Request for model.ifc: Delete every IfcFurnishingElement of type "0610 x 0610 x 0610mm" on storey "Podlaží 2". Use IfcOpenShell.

First a look at what the model holds.

```python
import ifcopenshell
import ifcopenshell.util.element

model = ifcopenshell.open("model.ifc")
print(model.schema)
storey = next(s for s in model.by_type("IfcBuildingStorey") if s.Name == "Podlaží 2")
furniture = [e for e in ifcopenshell.util.element.get_decomposition(storey) if e.is_a("IfcFurnishingElement")]
seen = {}
for e in furniture:
    element_type = ifcopenshell.util.element.get_type(e)
    name = element_type.Name if element_type not in (None, e) else None
    seen[name] = seen.get(name, 0) + 1
for name, count in sorted(seen.items(), key=str):
    print(count, "x", name)
```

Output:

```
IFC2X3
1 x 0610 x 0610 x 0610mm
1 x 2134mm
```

```python
import ifcopenshell
import ifcopenshell.api.root
import ifcopenshell.util.element

model = ifcopenshell.open("model.ifc")

storey = next(s for s in model.by_type("IfcBuildingStorey") if s.Name == "Podlaží 2")
furniture = [e for e in ifcopenshell.util.element.get_decomposition(storey) if e.is_a("IfcFurnishingElement")]
targets = [e for e in furniture if (t := ifcopenshell.util.element.get_type(e)) not in (None, e) and t.Name == "0610 x 0610 x 0610mm"]

for e in targets:
    ifcopenshell.api.root.remove_product(model, product=e)
print(len(targets), "removed")

model.write("model_rev.ifc")
```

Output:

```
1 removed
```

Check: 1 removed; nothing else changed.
